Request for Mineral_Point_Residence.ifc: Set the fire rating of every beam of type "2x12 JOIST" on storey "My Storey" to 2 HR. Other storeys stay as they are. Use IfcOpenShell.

First a look at what the model holds.

```python
import ifcopenshell
import ifcopenshell.util.element

model = ifcopenshell.open("Mineral_Point_Residence.ifc")
print(model.schema)
storey = next(s for s in model.by_type("IfcBuildingStorey") if s.Name == "My Storey")
beams = [e for e in ifcopenshell.util.element.get_decomposition(storey) if e.is_a("IfcBeam")]
seen = {}
for e in beams:
    element_type = ifcopenshell.util.element.get_type(e)
    key = (element_type.Name if element_type != e and element_type else None, ifcopenshell.util.element.get_pset(e, "Pset_BeamCommon", "FireRating"))
    seen[key] = seen.get(key, 0) + 1
for (name, value), count in sorted(seen.items(), key=str):
    print(count, "x", name, "|", value)
```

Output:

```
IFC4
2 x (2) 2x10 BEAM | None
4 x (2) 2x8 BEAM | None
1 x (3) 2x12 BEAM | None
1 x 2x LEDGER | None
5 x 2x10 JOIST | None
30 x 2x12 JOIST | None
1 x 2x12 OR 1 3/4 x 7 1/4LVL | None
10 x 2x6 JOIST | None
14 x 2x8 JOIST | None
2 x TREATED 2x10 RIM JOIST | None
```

```python
import ifcopenshell
import ifcopenshell.api.pset
import ifcopenshell.util.element

model = ifcopenshell.open("Mineral_Point_Residence.ifc")

storey = next(s for s in model.by_type("IfcBuildingStorey") if s.Name == "My Storey")
beams = [e for e in ifcopenshell.util.element.get_decomposition(storey) if e.is_a("IfcBeam")]

count = 0
for e in beams:
    element_type = ifcopenshell.util.element.get_type(e)
    if element_type in (None, e) or element_type.Name != "2x12 JOIST":
        continue
    # add_pset returns the element's existing set when there is one.
    pset = ifcopenshell.api.pset.add_pset(model, product=e, name="Pset_BeamCommon")
    ifcopenshell.api.pset.edit_pset(model, pset=pset, properties={"FireRating": "2 HR"})
    count += 1

print(count, "beams updated")

model.write("Mineral_Point_Residence_rev.ifc")
```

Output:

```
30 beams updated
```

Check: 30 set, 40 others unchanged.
